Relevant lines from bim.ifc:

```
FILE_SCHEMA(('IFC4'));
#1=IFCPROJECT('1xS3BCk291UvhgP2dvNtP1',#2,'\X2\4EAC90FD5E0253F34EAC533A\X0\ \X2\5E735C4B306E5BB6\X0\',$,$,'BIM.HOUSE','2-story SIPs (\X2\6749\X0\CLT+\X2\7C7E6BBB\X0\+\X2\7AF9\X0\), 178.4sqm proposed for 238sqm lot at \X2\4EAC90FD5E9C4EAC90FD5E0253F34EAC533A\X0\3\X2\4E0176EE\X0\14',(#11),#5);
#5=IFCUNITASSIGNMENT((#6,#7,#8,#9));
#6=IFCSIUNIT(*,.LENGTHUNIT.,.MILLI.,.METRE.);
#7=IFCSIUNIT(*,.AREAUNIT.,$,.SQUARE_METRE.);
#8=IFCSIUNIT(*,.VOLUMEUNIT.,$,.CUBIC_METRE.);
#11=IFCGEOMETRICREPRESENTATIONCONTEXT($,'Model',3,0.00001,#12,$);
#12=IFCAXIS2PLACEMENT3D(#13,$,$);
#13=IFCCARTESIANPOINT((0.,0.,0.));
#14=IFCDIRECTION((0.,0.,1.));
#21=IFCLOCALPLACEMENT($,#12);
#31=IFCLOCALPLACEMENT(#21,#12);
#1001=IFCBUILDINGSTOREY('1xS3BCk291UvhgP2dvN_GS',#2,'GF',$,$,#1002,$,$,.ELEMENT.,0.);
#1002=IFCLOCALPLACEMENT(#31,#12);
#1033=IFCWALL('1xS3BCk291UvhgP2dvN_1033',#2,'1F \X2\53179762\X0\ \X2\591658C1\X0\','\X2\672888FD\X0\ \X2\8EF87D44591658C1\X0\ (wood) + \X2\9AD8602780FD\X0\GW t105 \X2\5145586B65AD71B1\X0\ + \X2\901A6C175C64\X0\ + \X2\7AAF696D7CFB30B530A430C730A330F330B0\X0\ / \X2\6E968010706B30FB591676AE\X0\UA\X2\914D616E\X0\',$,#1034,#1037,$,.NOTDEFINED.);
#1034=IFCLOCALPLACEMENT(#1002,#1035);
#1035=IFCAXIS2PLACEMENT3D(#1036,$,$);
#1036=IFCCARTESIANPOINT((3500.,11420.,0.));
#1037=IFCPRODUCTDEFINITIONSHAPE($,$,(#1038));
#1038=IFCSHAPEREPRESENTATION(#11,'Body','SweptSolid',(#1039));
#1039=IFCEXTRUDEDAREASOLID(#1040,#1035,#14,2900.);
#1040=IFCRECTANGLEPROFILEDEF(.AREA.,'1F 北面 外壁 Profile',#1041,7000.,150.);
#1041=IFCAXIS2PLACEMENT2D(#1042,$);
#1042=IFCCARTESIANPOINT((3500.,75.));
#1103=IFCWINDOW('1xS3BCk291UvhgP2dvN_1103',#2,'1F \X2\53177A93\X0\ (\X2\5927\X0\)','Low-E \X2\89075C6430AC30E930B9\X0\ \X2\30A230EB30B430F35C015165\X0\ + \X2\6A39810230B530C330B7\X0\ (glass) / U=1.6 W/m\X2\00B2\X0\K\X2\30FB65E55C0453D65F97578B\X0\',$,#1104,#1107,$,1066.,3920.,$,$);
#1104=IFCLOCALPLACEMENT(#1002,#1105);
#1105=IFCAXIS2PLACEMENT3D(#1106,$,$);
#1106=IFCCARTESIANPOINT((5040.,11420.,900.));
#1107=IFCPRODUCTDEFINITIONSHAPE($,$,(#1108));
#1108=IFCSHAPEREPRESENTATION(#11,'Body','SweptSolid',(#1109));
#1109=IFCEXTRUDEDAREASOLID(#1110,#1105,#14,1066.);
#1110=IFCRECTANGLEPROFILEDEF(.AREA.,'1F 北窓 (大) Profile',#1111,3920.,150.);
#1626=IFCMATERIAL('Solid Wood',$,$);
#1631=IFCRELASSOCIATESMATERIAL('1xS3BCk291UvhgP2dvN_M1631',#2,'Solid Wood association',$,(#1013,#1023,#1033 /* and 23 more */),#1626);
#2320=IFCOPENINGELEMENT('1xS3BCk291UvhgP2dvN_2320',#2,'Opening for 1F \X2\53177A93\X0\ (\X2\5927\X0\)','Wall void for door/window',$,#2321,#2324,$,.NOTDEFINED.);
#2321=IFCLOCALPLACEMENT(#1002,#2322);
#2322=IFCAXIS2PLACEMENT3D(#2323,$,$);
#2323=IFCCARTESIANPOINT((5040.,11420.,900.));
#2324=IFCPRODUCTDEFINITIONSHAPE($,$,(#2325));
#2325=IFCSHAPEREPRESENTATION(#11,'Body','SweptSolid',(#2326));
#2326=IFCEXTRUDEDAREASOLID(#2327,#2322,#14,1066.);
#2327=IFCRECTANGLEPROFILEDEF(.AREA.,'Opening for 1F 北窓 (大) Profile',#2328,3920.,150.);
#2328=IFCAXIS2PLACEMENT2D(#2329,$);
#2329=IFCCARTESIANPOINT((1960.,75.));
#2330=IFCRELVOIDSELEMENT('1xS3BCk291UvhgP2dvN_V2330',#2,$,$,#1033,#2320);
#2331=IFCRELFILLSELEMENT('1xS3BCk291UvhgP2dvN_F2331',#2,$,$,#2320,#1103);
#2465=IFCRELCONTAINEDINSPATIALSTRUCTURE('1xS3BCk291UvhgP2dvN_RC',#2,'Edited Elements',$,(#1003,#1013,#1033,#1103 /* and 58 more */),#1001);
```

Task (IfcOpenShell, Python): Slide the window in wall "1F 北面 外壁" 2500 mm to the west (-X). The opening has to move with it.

```python
import ifcopenshell
import ifcopenshell.api.geometry
import ifcopenshell.util.placement
import ifcopenshell.util.unit

model = ifcopenshell.open("bim.ifc")
unit_scale = ifcopenshell.util.unit.calculate_unit_scale(model)

window = model.by_guid("1xS3BCk291UvhgP2dvN_1103")
opening = window.FillsVoids[0].RelatingOpeningElement
wall = opening.VoidsElements[0].RelatingBuildingElement

wall_matrix = ifcopenshell.util.placement.get_local_placement(wall.ObjectPlacement)
shift = wall_matrix[:3, 0] * -2.5 / unit_scale
before = ifcopenshell.util.placement.get_local_placement(window.ObjectPlacement)[:3, 3].copy()

# The window is not placed relative to its opening, so move both.
for product in (opening, window):
    matrix = ifcopenshell.util.placement.get_local_placement(product.ObjectPlacement)
    matrix[:3, 3] += shift
    ifcopenshell.api.geometry.edit_object_placement(model, product=product, matrix=matrix, is_si=False)

after = ifcopenshell.util.placement.get_local_placement(window.ObjectPlacement)[:3, 3]
print("window moved by", (after - before).round(3) + 0.0)

model.write("bim_edited.ifc")
```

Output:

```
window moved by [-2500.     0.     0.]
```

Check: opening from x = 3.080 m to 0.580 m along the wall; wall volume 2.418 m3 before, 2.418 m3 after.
